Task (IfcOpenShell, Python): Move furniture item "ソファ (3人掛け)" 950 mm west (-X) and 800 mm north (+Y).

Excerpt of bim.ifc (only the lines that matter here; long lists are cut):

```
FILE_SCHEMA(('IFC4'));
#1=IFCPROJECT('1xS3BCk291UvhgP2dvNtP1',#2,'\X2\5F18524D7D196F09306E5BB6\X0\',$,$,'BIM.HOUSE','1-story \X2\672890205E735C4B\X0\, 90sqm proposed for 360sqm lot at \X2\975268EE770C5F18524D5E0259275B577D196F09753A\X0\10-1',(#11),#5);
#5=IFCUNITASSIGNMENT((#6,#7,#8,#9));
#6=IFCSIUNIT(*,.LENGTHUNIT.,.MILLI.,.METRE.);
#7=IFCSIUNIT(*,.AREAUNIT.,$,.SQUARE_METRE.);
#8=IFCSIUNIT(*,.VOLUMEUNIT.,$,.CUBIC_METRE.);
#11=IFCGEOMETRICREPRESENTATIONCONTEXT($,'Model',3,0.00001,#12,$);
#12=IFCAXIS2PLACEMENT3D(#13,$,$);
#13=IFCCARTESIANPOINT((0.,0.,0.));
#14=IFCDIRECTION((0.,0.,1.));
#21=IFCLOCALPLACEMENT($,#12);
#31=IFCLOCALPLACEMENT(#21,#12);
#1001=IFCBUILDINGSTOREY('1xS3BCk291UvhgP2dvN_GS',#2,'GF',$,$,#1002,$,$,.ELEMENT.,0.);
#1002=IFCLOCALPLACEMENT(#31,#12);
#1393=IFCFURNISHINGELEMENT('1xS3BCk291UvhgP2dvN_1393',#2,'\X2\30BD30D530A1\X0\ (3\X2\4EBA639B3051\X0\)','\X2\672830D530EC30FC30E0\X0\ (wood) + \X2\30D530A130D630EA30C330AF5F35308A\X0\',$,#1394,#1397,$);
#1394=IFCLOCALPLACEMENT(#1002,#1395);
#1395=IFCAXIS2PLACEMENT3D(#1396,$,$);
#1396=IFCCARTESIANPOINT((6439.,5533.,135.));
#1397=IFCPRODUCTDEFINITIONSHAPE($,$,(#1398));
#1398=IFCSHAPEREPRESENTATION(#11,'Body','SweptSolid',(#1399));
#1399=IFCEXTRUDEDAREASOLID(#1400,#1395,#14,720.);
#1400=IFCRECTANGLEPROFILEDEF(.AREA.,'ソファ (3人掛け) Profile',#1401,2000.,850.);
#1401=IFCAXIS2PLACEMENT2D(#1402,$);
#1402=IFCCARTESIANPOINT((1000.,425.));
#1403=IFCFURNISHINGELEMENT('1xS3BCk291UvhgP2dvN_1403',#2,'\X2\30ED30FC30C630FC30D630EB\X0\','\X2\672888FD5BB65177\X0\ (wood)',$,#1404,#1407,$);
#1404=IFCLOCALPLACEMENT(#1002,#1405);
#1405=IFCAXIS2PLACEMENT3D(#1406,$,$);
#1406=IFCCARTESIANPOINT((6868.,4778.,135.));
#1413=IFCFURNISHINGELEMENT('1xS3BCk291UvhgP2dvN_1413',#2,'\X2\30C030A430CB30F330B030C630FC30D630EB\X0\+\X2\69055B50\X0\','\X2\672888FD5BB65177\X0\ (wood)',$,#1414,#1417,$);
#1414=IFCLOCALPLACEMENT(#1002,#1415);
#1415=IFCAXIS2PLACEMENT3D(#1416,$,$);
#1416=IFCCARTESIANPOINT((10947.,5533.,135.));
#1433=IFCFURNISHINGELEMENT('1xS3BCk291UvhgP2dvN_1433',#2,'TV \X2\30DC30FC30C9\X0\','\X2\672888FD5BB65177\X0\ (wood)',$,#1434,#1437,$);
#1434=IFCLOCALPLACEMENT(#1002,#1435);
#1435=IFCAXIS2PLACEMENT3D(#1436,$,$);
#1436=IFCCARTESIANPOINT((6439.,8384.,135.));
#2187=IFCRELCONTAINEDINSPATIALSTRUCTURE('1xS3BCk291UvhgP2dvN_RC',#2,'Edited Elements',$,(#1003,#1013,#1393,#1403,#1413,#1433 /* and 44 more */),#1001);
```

```python
import ifcopenshell
import ifcopenshell.api.geometry
import ifcopenshell.util.placement

model = ifcopenshell.open("bim.ifc")

item = model.by_guid("1xS3BCk291UvhgP2dvN_1393")
matrix = ifcopenshell.util.placement.get_local_placement(item.ObjectPlacement)
matrix[0, 3] -= 950.0
matrix[1, 3] += 800.0
ifcopenshell.api.geometry.edit_object_placement(model, product=item, matrix=matrix, is_si=False)

print(ifcopenshell.util.placement.get_local_placement(item.ObjectPlacement).round(3) + 0.0)

model.write("bim_rev.ifc")
```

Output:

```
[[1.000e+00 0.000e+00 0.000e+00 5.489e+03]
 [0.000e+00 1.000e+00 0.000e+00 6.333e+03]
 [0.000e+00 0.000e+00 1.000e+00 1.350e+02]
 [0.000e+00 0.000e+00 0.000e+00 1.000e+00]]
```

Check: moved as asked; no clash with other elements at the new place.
